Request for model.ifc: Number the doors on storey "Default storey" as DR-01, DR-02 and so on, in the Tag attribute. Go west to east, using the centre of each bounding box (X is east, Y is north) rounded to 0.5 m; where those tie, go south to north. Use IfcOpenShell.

First a look at what the model holds.

```python
import ifcopenshell
import ifcopenshell.util.element
import ifcopenshell.util.placement

model = ifcopenshell.open("model.ifc")
print(model.schema)
storey = next(s for s in model.by_type("IfcBuildingStorey") if s.Name == "Default storey")
doors = [e for e in ifcopenshell.util.element.get_decomposition(storey) if e.is_a("IfcDoor")]
for e in sorted(doors, key=lambda e: e.id()):
    origin = ifcopenshell.util.placement.get_local_placement(e.ObjectPlacement)[:3, 3]
    print(e.id(), e.Tag, e.Name, origin.round(2) + 0.0, sep=" | ")
```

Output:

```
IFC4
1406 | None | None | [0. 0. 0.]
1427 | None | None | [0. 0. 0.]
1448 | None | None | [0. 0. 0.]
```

```python
import ifcopenshell
import ifcopenshell.geom
import ifcopenshell.util.element
import ifcopenshell.util.shape

model = ifcopenshell.open("model.ifc")
settings = ifcopenshell.geom.settings()
settings.set("use-world-coords", True)


def centre(element):
    shape = ifcopenshell.geom.create_shape(settings, element)
    return ifcopenshell.util.shape.get_bbox_centroid(shape.geometry)


storey = next(s for s in model.by_type("IfcBuildingStorey") if s.Name == "Default storey")
doors = [e for e in ifcopenshell.util.element.get_decomposition(storey) if e.is_a("IfcDoor")]

# Insertion points can sit at a corner or the storey origin, so sort by the geometry (in metres).
centres = {e: centre(e) for e in doors}
doors.sort(key=lambda e: (round(centres[e][0] / 0.5), centres[e][1]))

for i, e in enumerate(doors, start=1):
    number = f"DR-{i:02d}"
    e.Tag = number
    print(e.id(), number)

model.write("model_rev.ifc")
```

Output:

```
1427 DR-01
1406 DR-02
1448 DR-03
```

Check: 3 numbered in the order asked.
